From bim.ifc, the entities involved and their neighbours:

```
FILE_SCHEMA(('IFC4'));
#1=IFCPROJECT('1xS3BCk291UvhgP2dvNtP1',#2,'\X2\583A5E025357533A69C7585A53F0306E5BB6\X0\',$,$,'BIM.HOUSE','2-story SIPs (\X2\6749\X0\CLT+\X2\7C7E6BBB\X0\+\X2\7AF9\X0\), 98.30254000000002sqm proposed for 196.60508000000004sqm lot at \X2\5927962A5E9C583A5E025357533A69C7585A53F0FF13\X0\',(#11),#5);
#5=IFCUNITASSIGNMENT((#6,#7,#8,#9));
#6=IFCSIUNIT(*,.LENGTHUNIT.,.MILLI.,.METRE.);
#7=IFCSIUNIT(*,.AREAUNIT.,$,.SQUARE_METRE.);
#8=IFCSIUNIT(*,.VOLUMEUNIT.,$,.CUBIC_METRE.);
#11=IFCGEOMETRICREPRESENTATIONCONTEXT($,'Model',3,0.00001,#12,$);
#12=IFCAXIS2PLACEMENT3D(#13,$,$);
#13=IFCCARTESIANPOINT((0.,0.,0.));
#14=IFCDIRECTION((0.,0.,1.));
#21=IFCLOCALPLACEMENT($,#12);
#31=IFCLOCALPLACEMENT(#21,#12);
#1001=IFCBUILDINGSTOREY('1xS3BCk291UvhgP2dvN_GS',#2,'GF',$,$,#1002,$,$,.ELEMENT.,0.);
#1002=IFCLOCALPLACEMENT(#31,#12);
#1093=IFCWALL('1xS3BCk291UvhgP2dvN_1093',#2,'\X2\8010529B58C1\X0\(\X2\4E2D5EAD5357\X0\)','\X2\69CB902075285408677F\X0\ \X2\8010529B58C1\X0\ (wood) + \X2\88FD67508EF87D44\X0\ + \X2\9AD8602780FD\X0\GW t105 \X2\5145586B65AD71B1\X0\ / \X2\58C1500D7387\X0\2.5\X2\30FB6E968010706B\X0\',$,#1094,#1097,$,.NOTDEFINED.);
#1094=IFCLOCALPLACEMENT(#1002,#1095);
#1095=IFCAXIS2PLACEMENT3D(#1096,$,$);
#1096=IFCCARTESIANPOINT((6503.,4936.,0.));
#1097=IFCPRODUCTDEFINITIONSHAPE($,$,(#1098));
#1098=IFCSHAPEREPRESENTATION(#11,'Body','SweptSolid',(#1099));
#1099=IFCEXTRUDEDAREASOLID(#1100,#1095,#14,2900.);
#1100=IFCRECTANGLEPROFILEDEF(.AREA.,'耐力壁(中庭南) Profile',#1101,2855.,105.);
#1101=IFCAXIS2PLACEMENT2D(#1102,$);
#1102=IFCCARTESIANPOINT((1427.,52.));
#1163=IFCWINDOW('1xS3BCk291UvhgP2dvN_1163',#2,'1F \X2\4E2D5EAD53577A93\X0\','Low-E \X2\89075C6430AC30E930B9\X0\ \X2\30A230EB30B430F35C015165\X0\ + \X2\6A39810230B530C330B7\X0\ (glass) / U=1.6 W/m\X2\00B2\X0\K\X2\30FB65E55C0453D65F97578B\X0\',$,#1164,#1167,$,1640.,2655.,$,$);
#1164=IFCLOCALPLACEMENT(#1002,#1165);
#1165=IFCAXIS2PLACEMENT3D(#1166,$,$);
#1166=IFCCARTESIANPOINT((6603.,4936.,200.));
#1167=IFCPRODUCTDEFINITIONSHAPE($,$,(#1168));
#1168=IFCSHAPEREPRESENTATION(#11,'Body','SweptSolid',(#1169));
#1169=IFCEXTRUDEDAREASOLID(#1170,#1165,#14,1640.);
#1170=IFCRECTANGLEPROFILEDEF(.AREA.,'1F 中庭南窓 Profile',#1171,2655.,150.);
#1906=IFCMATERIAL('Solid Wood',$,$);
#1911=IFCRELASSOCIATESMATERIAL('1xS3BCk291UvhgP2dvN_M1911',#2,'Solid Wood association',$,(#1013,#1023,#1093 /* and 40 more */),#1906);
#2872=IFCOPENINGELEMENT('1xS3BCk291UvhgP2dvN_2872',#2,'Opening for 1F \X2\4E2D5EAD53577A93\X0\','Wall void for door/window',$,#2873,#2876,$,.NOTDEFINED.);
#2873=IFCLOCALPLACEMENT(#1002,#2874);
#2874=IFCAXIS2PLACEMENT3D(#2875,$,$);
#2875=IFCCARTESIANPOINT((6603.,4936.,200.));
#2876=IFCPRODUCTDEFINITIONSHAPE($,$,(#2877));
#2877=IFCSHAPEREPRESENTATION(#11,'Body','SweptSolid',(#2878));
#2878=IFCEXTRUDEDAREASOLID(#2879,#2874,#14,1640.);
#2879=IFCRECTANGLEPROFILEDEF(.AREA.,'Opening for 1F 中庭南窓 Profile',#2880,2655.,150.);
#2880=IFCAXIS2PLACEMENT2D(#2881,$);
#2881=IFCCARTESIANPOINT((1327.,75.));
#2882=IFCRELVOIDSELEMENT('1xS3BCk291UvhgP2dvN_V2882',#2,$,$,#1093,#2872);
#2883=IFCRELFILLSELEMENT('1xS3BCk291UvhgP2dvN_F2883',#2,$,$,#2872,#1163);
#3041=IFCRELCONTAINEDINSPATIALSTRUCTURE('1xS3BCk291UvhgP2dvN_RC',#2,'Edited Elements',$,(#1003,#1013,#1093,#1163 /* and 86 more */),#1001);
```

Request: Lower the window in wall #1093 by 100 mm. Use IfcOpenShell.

```python
import numpy as np
import ifcopenshell
import ifcopenshell.api.geometry
import ifcopenshell.util.placement
import ifcopenshell.util.unit

model = ifcopenshell.open("bim.ifc")
unit_scale = ifcopenshell.util.unit.calculate_unit_scale(model)

window = model.by_guid("1xS3BCk291UvhgP2dvN_1163")
opening = window.FillsVoids[0].RelatingOpeningElement
dz = -0.1 / unit_scale

shift = np.array([0.0, 0.0, dz])
# The window is not placed relative to its opening, so move both.
for product in (opening, window):
    matrix = ifcopenshell.util.placement.get_local_placement(product.ObjectPlacement)
    matrix[:3, 3] += shift
    ifcopenshell.api.geometry.edit_object_placement(model, product=product, matrix=matrix, is_si=False)

print(f"moved by {dz * unit_scale:+.3f} m")

model.write("bim_v2.ifc")
```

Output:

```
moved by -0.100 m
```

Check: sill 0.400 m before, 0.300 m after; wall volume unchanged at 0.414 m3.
